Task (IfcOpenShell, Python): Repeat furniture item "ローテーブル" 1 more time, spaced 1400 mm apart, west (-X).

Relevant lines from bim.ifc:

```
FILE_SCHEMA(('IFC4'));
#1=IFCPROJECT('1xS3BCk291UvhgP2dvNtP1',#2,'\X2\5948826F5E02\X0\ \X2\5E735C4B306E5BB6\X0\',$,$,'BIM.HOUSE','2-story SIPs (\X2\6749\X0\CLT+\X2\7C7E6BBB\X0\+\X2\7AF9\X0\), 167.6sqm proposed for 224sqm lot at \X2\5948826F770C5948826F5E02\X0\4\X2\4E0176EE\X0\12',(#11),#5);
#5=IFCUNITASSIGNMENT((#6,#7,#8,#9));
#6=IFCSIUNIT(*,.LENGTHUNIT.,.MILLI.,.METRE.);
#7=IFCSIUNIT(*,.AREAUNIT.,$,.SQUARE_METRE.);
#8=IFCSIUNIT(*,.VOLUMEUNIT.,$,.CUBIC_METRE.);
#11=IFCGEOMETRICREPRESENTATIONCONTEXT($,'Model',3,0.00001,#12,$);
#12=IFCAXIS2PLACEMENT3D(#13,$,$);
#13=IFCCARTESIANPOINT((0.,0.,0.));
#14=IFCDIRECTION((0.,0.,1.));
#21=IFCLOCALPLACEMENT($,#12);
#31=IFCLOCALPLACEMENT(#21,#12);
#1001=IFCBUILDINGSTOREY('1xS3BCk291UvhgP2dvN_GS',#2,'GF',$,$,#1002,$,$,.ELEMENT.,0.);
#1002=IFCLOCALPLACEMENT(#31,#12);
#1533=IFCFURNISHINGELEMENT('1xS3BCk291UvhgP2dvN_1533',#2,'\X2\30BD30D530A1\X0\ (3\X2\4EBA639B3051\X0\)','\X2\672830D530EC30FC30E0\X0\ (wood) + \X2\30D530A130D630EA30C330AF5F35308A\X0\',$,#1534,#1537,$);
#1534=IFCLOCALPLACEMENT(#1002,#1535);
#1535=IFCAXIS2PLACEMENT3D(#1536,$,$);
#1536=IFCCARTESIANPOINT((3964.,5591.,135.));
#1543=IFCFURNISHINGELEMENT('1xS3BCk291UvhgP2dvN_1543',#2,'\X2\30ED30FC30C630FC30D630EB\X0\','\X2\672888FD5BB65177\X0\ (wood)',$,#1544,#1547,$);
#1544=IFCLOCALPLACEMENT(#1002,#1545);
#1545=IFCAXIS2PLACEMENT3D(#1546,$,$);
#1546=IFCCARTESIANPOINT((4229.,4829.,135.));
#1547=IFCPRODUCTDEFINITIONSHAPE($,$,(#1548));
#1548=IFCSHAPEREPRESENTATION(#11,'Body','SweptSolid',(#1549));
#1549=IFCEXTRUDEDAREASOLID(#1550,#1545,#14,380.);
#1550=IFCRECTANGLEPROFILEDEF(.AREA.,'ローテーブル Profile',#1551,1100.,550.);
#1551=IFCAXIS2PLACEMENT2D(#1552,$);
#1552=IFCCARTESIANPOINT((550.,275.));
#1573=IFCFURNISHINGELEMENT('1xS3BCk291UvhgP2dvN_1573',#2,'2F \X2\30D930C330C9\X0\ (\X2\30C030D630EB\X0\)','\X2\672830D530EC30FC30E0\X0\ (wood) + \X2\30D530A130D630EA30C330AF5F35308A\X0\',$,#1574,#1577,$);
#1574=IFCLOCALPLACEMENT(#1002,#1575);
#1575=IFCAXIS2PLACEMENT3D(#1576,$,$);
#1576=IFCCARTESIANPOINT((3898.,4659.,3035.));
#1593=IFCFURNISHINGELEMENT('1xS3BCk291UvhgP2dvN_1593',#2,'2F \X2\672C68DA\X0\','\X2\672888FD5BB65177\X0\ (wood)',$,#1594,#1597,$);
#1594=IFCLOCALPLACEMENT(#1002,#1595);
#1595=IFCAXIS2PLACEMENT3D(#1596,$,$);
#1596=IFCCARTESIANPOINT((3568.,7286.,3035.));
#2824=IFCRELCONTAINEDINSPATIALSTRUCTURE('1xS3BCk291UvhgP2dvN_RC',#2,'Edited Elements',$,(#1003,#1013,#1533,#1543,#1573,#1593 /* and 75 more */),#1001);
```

```python
import numpy as np
import ifcopenshell
import ifcopenshell.api.geometry
import ifcopenshell.api.root
import ifcopenshell.util.element
import ifcopenshell.util.placement

model = ifcopenshell.open("bim.ifc")


def reuse_history(source, copy):
    """copy_class also copies each property set's owner history, people and application; keep the originals."""
    for rel in copy.IsDefinedBy:
        if rel.is_a("IfcRelDefinesByProperties") and (history := rel.RelatingPropertyDefinition.OwnerHistory):
            rel.RelatingPropertyDefinition.OwnerHistory = source.OwnerHistory
            ifcopenshell.util.element.remove_deep2(model, history)


source = model.by_guid("1xS3BCk291UvhgP2dvN_1543")
base = ifcopenshell.util.placement.get_local_placement(source.ObjectPlacement)
step = np.array([-1.0, 0.0, 0.0]) * 1400.0

for i in range(1, 2):
    copy = ifcopenshell.api.root.copy_class(model, product=source)
    copy.Representation = ifcopenshell.util.element.copy_deep(
        model, source.Representation, exclude=["IfcGeometricRepresentationContext", "IfcRepresentationMap"]
    )
    reuse_history(source, copy)
    matrix = base.copy()
    matrix[:3, 3] += i * step
    print("added at", matrix[:3, 3].round(3) + 0.0)
    ifcopenshell.api.geometry.edit_object_placement(model, product=copy, matrix=matrix, is_si=False)

model.write("bim_rev.ifc")
```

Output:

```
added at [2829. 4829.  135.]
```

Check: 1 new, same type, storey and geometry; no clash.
